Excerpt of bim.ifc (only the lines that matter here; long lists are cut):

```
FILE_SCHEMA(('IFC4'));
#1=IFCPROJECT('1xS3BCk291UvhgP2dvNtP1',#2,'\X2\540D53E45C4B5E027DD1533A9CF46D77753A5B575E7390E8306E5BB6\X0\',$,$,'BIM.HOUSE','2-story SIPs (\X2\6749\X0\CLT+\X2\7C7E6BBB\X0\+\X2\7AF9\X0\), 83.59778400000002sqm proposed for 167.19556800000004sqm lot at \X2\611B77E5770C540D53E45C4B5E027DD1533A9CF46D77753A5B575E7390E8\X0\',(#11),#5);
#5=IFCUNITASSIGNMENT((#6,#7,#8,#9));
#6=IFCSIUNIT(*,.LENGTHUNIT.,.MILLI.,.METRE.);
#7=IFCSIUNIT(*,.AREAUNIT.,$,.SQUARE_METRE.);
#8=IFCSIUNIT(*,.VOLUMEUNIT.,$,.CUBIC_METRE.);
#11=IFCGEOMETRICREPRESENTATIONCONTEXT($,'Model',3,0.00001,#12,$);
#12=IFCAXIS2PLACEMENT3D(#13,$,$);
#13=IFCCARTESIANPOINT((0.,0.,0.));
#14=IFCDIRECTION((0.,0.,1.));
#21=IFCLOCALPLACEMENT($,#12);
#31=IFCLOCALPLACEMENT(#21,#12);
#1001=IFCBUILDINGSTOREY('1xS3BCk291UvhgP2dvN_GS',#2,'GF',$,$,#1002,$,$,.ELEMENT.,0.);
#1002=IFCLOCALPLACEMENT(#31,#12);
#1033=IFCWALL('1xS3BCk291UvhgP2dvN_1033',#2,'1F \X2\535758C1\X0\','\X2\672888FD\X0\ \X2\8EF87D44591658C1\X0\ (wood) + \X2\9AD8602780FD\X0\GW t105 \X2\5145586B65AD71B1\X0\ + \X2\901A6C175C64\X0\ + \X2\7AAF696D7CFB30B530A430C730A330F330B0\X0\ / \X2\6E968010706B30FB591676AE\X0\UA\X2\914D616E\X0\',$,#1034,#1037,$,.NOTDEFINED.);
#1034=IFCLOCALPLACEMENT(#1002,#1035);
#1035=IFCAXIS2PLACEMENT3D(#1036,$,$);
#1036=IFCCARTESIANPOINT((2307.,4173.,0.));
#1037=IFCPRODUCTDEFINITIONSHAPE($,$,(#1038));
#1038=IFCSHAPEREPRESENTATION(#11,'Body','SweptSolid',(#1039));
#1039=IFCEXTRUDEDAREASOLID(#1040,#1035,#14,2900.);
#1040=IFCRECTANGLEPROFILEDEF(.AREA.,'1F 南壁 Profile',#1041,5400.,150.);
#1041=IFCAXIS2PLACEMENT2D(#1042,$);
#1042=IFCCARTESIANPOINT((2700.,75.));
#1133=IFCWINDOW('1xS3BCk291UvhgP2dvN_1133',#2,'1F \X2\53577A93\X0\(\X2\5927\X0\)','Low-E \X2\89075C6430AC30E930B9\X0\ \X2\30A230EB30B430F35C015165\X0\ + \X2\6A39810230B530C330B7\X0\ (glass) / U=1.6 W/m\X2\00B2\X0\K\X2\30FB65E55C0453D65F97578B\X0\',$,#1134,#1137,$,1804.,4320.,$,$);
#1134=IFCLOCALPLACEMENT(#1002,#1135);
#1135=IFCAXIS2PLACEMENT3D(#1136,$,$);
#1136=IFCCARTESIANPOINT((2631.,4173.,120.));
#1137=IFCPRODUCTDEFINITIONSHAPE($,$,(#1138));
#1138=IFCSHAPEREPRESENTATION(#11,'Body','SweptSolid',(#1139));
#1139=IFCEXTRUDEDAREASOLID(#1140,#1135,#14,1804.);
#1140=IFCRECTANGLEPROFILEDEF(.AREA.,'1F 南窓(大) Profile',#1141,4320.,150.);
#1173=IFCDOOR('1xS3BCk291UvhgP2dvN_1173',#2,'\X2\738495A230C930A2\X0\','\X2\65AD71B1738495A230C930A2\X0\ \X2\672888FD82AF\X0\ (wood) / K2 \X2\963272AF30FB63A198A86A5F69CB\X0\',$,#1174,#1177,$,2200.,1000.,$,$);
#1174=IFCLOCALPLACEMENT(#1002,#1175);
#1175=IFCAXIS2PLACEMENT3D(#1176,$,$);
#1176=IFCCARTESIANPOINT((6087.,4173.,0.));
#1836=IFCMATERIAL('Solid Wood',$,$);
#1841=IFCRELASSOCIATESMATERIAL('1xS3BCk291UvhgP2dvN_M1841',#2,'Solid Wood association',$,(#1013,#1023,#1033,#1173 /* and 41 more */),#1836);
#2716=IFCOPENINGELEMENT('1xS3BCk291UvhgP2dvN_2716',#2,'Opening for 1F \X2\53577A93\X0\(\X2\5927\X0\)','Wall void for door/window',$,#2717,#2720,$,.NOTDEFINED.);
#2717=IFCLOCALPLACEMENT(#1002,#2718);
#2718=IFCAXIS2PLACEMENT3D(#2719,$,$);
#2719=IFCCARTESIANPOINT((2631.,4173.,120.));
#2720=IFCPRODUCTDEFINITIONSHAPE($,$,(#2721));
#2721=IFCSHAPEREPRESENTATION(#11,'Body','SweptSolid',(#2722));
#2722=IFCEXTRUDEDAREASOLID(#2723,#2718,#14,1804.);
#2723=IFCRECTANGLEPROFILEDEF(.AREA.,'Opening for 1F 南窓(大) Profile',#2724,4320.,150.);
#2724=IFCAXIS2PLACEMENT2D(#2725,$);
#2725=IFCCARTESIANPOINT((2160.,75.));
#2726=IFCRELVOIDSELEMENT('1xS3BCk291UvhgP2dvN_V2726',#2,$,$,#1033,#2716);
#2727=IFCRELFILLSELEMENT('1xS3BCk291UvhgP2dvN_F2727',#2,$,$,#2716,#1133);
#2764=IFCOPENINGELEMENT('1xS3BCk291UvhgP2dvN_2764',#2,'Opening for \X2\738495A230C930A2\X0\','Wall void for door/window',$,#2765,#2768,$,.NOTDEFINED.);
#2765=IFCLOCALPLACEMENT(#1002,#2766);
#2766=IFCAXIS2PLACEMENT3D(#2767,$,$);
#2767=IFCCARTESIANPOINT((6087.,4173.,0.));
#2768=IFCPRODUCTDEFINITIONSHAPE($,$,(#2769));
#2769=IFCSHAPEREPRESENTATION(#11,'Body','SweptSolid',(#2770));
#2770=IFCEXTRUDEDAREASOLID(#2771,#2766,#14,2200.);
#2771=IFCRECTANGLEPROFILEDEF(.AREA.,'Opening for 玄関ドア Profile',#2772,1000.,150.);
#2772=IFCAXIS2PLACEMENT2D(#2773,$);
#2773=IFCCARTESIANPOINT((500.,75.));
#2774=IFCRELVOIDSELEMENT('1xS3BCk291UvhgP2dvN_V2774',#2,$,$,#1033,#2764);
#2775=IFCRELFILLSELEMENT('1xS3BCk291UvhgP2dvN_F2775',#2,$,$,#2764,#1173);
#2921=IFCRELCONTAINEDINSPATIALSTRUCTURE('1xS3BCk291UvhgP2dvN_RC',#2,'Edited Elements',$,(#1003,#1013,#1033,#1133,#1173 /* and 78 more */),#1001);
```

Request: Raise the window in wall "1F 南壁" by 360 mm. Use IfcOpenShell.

```python
import numpy as np
import ifcopenshell
import ifcopenshell.api.geometry
import ifcopenshell.util.placement
import ifcopenshell.util.unit

model = ifcopenshell.open("bim.ifc")
unit_scale = ifcopenshell.util.unit.calculate_unit_scale(model)

window = model.by_guid("1xS3BCk291UvhgP2dvN_1133")
opening = window.FillsVoids[0].RelatingOpeningElement
dz = 0.36 / unit_scale

shift = np.array([0.0, 0.0, dz])
# The window is not placed relative to its opening, so move both.
for product in (opening, window):
    matrix = ifcopenshell.util.placement.get_local_placement(product.ObjectPlacement)
    matrix[:3, 3] += shift
    ifcopenshell.api.geometry.edit_object_placement(model, product=product, matrix=matrix, is_si=False)

print(f"moved by {dz * unit_scale:+.3f} m")

model.write("bim_rev.ifc")
```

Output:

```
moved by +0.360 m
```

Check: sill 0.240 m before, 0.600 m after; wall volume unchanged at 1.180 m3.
